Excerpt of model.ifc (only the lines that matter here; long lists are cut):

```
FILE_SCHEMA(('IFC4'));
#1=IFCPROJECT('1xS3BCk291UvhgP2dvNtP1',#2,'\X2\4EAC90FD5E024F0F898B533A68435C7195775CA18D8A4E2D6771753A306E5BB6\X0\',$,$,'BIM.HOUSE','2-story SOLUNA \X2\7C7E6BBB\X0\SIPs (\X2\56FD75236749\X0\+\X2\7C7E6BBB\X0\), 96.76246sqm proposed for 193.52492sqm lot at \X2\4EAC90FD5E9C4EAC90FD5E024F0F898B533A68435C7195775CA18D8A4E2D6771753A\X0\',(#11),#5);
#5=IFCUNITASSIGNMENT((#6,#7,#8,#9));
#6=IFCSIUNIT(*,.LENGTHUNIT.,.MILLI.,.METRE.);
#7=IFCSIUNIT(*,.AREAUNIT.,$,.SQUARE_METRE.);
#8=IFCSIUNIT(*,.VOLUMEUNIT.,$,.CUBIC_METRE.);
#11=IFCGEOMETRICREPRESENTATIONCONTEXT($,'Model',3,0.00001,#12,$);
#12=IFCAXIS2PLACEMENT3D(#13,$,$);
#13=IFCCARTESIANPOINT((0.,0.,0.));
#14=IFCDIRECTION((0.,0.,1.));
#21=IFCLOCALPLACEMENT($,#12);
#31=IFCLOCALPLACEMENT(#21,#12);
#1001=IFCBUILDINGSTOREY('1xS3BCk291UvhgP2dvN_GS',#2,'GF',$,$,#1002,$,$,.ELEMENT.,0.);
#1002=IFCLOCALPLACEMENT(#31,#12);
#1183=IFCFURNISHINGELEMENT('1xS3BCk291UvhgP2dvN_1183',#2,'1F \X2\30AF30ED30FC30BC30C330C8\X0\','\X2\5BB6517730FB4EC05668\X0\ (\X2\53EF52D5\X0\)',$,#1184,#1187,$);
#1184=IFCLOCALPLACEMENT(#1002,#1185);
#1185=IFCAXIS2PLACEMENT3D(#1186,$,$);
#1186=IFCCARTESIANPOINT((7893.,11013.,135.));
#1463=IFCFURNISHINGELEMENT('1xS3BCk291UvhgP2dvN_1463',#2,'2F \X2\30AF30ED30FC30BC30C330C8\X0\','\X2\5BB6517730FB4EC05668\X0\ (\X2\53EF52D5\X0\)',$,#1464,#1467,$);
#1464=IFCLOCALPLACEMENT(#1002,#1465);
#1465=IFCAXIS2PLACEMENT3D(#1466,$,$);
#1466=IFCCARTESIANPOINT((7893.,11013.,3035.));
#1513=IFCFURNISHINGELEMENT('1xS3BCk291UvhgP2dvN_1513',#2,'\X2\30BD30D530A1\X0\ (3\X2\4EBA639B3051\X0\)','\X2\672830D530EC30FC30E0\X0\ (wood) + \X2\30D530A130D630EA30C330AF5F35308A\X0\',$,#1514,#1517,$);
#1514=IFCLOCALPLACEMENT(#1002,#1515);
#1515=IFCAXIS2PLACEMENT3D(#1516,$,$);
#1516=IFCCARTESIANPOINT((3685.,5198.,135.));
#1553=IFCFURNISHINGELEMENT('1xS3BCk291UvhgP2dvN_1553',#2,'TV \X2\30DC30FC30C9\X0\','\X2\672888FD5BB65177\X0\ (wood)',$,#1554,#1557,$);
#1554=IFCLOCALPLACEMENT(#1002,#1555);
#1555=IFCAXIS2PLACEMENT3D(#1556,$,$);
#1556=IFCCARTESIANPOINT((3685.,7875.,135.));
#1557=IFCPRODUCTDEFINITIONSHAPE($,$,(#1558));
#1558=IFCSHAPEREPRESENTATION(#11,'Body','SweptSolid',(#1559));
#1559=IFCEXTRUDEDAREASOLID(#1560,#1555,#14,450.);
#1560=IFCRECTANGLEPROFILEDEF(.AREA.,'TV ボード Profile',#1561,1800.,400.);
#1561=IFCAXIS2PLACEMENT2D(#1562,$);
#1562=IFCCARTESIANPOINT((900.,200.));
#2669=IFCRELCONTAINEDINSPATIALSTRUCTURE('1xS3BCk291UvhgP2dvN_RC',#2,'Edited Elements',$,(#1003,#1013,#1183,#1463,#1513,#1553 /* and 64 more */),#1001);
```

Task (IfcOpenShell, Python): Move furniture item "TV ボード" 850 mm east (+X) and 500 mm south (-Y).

```python
import ifcopenshell
import ifcopenshell.api.geometry
import ifcopenshell.util.placement
import ifcopenshell.util.unit

model = ifcopenshell.open("model.ifc")
unit_scale = ifcopenshell.util.unit.calculate_unit_scale(model)

item = model.by_guid("1xS3BCk291UvhgP2dvN_1553")
matrix = ifcopenshell.util.placement.get_local_placement(item.ObjectPlacement)
matrix[0, 3] += 0.85 / unit_scale
matrix[1, 3] -= 0.5 / unit_scale
ifcopenshell.api.geometry.edit_object_placement(model, product=item, matrix=matrix, is_si=False)

print(ifcopenshell.util.placement.get_local_placement(item.ObjectPlacement).round(3) + 0.0)

model.write("model_updated.ifc")
```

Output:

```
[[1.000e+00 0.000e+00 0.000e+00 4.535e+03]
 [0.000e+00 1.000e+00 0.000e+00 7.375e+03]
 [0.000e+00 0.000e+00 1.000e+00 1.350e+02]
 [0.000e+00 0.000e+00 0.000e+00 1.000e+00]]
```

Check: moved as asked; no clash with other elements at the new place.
